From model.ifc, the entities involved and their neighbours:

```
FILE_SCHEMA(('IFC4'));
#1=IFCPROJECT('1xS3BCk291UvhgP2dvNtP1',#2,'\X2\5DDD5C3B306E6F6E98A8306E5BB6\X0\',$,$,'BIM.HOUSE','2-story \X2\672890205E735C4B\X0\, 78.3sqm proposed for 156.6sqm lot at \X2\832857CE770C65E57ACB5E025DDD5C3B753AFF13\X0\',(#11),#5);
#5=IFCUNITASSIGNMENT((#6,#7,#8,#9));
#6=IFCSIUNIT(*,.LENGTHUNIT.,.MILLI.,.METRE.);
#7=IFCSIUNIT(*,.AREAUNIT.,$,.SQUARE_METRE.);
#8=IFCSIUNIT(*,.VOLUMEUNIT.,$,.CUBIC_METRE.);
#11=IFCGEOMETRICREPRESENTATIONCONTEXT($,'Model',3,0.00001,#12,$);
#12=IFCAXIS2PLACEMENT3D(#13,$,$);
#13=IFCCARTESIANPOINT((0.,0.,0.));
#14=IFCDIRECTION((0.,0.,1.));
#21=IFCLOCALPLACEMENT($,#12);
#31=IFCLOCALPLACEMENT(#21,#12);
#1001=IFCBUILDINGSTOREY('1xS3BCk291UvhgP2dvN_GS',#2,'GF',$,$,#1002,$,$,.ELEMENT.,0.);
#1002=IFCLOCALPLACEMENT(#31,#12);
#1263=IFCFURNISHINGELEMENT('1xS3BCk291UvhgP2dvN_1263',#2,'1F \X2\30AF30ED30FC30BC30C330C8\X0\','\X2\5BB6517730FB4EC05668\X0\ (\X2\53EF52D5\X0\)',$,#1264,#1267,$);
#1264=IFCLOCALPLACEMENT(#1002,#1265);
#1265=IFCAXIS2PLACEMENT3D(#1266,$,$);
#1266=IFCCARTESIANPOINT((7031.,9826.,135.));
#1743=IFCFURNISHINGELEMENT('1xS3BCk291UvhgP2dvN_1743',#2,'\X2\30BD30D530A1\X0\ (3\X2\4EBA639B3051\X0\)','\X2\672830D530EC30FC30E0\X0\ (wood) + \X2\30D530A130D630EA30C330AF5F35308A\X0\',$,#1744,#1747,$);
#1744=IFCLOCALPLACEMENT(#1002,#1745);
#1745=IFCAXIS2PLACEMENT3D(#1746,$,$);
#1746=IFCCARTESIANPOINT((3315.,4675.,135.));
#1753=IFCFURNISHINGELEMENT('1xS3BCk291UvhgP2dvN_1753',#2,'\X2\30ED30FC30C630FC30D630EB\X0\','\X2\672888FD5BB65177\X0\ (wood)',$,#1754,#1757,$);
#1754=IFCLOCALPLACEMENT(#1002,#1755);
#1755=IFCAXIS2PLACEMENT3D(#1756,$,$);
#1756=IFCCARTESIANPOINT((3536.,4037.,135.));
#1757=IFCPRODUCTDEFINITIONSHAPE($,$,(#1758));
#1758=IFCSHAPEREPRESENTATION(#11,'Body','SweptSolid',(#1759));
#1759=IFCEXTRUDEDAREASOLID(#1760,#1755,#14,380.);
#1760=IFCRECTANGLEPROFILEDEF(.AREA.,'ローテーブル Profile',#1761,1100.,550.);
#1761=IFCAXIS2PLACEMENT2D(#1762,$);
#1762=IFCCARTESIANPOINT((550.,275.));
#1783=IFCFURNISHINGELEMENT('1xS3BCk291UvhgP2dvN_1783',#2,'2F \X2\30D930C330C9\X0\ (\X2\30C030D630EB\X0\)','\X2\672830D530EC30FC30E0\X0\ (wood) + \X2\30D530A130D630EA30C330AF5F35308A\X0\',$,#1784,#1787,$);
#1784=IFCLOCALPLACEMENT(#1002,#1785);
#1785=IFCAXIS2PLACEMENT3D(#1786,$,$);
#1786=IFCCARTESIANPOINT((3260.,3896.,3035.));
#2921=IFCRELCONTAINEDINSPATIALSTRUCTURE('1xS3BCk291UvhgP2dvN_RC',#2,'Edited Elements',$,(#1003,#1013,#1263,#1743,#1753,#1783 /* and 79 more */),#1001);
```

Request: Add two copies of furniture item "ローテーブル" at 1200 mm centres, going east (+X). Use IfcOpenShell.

```python
import numpy as np
import ifcopenshell
import ifcopenshell.api.geometry
import ifcopenshell.api.root
import ifcopenshell.util.element
import ifcopenshell.util.placement
import ifcopenshell.util.unit

model = ifcopenshell.open("model.ifc")
unit_scale = ifcopenshell.util.unit.calculate_unit_scale(model)


def reuse_history(source, copy):
    """copy_class also copies each property set's owner history, people and application; keep the originals."""
    for rel in copy.IsDefinedBy:
        if rel.is_a("IfcRelDefinesByProperties") and (history := rel.RelatingPropertyDefinition.OwnerHistory):
            rel.RelatingPropertyDefinition.OwnerHistory = source.OwnerHistory
            ifcopenshell.util.element.remove_deep2(model, history)


source = model.by_guid("1xS3BCk291UvhgP2dvN_1753")
base = ifcopenshell.util.placement.get_local_placement(source.ObjectPlacement)
step = np.array([1.0, 0.0, 0.0]) * 1.2 / unit_scale

for i in range(1, 3):
    copy = ifcopenshell.api.root.copy_class(model, product=source)
    copy.Representation = ifcopenshell.util.element.copy_deep(
        model, source.Representation, exclude=["IfcGeometricRepresentationContext", "IfcRepresentationMap"]
    )
    reuse_history(source, copy)
    matrix = base.copy()
    matrix[:3, 3] += i * step
    print("added at", matrix[:3, 3].round(3) + 0.0)
    ifcopenshell.api.geometry.edit_object_placement(model, product=copy, matrix=matrix, is_si=False)

model.write("model_edited.ifc")
```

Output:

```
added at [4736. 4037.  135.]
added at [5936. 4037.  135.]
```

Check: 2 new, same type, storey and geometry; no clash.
